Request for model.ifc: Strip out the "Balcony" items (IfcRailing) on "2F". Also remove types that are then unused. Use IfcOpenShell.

First a look at what the model holds.

```python
import ifcopenshell
import ifcopenshell.util.element

model = ifcopenshell.open("model.ifc")
print(model.schema)
storey = next(s for s in model.by_type("IfcBuildingStorey") if s.Name == "2F")
railings = [e for e in ifcopenshell.util.element.get_decomposition(storey) if e.is_a("IfcRailing")]
seen = {}
for e in railings:
    element_type = ifcopenshell.util.element.get_type(e)
    name = element_type.Name if element_type not in (None, e) else None
    seen[name] = seen.get(name, 0) + 1
for name, count in sorted(seen.items(), key=str):
    print(count, "x", name)
```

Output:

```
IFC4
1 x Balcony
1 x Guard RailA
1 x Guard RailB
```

```python
import ifcopenshell
import ifcopenshell.api.root
import ifcopenshell.util.element

model = ifcopenshell.open("model.ifc")

storey = next(s for s in model.by_type("IfcBuildingStorey") if s.Name == "2F")
railings = [e for e in ifcopenshell.util.element.get_decomposition(storey) if e.is_a("IfcRailing")]
targets = [e for e in railings if (t := ifcopenshell.util.element.get_type(e)) not in (None, e) and t.Name == "Balcony"]
types = {ifcopenshell.util.element.get_type(e) for e in targets} - {None, *targets}

for e in targets:
    ifcopenshell.api.root.remove_product(model, product=e)
print(len(targets), "removed")

unused = [t for t in types if not ifcopenshell.util.element.get_types(t)]
for t in unused:
    ifcopenshell.api.root.remove_product(model, product=t)
print(len(unused), "unused types removed")

model.write("model_rev.ifc")
```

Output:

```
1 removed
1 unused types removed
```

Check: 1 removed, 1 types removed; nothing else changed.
